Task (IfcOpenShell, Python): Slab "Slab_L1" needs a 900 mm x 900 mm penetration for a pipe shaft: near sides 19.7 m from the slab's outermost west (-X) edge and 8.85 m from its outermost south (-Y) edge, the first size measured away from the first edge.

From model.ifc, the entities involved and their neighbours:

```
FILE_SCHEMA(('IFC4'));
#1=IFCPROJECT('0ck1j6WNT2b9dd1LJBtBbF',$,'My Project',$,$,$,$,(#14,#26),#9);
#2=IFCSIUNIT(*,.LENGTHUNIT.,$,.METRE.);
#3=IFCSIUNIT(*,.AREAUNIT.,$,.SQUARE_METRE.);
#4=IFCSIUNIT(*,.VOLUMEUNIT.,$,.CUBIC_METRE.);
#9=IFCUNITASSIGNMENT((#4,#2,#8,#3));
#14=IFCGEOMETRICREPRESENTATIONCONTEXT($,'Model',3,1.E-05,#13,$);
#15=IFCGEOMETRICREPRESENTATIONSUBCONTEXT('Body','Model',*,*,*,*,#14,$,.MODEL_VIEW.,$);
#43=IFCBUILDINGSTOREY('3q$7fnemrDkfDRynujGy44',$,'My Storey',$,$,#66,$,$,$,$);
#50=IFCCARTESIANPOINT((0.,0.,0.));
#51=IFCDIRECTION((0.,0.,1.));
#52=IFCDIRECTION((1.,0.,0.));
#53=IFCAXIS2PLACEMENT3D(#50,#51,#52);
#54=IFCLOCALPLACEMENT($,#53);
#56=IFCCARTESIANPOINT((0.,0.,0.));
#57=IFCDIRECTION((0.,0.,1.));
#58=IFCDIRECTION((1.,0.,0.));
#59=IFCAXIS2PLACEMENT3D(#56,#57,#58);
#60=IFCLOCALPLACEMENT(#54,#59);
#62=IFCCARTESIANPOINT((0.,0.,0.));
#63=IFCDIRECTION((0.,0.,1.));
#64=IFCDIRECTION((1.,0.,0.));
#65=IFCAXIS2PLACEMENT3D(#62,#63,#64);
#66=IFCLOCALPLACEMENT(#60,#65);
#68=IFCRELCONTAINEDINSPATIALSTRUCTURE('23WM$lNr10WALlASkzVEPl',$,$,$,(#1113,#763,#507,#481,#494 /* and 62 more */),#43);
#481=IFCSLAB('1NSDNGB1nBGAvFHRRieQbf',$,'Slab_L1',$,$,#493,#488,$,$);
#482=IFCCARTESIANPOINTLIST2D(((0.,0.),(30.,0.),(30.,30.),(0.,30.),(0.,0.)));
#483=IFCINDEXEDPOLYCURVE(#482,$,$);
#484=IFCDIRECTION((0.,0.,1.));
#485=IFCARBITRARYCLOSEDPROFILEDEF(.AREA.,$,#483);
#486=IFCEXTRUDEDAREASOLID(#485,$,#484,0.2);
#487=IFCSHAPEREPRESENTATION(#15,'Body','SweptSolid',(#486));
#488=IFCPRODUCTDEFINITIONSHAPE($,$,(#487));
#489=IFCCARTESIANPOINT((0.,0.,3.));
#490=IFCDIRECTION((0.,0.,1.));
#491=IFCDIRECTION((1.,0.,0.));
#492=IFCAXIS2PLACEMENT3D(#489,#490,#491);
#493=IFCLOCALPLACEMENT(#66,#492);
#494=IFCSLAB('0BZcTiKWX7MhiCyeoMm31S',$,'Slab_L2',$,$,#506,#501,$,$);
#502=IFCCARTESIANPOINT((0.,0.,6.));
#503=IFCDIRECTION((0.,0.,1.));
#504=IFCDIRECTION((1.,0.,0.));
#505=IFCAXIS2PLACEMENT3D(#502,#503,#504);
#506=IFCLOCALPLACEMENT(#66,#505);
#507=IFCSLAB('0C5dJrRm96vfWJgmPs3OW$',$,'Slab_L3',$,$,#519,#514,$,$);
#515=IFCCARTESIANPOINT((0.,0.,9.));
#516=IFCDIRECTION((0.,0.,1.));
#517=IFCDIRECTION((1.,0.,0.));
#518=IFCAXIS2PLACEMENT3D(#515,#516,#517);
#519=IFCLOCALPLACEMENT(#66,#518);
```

```python
import numpy as np
import ifcopenshell
import ifcopenshell.api.feature
import ifcopenshell.api.geometry
import ifcopenshell.api.root
import ifcopenshell.geom
import ifcopenshell.util.placement
import ifcopenshell.util.representation
import ifcopenshell.util.shape
import ifcopenshell.util.unit

model = ifcopenshell.open("model.ifc")
unit_scale = ifcopenshell.util.unit.calculate_unit_scale(model)
settings = ifcopenshell.geom.settings()


def volume(element):
    """Net volume in cubic metres, openings subtracted."""
    shape = ifcopenshell.geom.create_shape(settings, element)
    return ifcopenshell.util.shape.get_volume(shape.geometry)


slab = model.by_guid("1NSDNGB1nBGAvFHRRieQbf")
before = volume(slab)

# Extent in the slab's own axes, in metres. The edges named are its -X and -Y sides.
slab_shape = ifcopenshell.geom.create_shape(settings, slab)
vertices = ifcopenshell.util.shape.get_vertices(slab_shape.geometry)
x_min, y_min, bottom = vertices.min(axis=0)
top = vertices[:, 2].max()

opening = ifcopenshell.api.root.create_entity(model, ifc_class="IfcOpeningElement", name="Pipe shaft opening", predefined_type="OPENING")
context = ifcopenshell.util.representation.get_context(model, "Model", "Body", "MODEL_VIEW")
width, depth = 0.9, 0.9
outline = [(0.0, 0.0), (width, 0.0), (width, depth), (0.0, depth), (0.0, 0.0)]
# Overshoot both faces by 50 mm so the cut is clean.
shape = ifcopenshell.api.geometry.add_slab_representation(
    model, context=context, depth=top - bottom + 0.1, polyline=outline
)
ifcopenshell.api.geometry.assign_representation(model, product=opening, representation=shape)

matrix = ifcopenshell.util.placement.get_local_placement(slab.ObjectPlacement)
matrix[:, 3] = matrix @ np.append(np.array([x_min + 19.7, y_min + 8.85, bottom - 0.05]) / unit_scale, 1.0)
ifcopenshell.api.geometry.edit_object_placement(model, product=opening, matrix=matrix, is_si=False)
ifcopenshell.api.feature.add_feature(model, feature=opening, element=slab)

after = volume(slab)

print(f"slab volume {before:.3f} -> {after:.3f} m3")

model.write("model_v2.ifc")
```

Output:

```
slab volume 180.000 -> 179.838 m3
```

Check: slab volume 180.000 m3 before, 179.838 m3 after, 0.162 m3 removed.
